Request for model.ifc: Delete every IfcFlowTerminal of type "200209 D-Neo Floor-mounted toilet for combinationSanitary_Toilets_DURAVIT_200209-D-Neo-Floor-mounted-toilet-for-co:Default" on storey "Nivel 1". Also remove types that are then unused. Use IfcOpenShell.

First a look at what the model holds.

```python
import ifcopenshell
import ifcopenshell.util.element

model = ifcopenshell.open("model.ifc")
print(model.schema)
storey = next(s for s in model.by_type("IfcBuildingStorey") if s.Name == "Nivel 1")
terminals = [e for e in ifcopenshell.util.element.get_decomposition(storey) if e.is_a("IfcFlowTerminal")]
seen = {}
for e in terminals:
    element_type = ifcopenshell.util.element.get_type(e)
    name = element_type.Name if element_type not in (None, e) else None
    seen[name] = seen.get(name, 0) + 1
for name, count in sorted(seen.items(), key=str):
    print(count, "x", name)
```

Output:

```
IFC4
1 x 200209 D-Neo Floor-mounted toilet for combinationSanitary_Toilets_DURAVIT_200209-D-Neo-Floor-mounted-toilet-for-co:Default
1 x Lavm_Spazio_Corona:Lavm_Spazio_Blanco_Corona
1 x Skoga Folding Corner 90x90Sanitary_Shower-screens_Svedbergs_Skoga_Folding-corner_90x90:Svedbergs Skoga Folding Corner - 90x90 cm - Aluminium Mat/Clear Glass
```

```python
import ifcopenshell
import ifcopenshell.api.root
import ifcopenshell.util.element

model = ifcopenshell.open("model.ifc")

storey = next(s for s in model.by_type("IfcBuildingStorey") if s.Name == "Nivel 1")
terminals = [e for e in ifcopenshell.util.element.get_decomposition(storey) if e.is_a("IfcFlowTerminal")]
targets = [e for e in terminals if (t := ifcopenshell.util.element.get_type(e)) not in (None, e) and t.Name == "200209 D-Neo Floor-mounted toilet for combinationSanitary_Toilets_DURAVIT_200209-D-Neo-Floor-mounted-toilet-for-co:Default"]
types = {ifcopenshell.util.element.get_type(e) for e in targets} - {None, *targets}

for e in targets:
    ifcopenshell.api.root.remove_product(model, product=e)
print(len(targets), "removed")

unused = [t for t in types if not ifcopenshell.util.element.get_types(t)]
for t in unused:
    ifcopenshell.api.root.remove_product(model, product=t)
print(len(unused), "unused types removed")

model.write("model-out.ifc")
```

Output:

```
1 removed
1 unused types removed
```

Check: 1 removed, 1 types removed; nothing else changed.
